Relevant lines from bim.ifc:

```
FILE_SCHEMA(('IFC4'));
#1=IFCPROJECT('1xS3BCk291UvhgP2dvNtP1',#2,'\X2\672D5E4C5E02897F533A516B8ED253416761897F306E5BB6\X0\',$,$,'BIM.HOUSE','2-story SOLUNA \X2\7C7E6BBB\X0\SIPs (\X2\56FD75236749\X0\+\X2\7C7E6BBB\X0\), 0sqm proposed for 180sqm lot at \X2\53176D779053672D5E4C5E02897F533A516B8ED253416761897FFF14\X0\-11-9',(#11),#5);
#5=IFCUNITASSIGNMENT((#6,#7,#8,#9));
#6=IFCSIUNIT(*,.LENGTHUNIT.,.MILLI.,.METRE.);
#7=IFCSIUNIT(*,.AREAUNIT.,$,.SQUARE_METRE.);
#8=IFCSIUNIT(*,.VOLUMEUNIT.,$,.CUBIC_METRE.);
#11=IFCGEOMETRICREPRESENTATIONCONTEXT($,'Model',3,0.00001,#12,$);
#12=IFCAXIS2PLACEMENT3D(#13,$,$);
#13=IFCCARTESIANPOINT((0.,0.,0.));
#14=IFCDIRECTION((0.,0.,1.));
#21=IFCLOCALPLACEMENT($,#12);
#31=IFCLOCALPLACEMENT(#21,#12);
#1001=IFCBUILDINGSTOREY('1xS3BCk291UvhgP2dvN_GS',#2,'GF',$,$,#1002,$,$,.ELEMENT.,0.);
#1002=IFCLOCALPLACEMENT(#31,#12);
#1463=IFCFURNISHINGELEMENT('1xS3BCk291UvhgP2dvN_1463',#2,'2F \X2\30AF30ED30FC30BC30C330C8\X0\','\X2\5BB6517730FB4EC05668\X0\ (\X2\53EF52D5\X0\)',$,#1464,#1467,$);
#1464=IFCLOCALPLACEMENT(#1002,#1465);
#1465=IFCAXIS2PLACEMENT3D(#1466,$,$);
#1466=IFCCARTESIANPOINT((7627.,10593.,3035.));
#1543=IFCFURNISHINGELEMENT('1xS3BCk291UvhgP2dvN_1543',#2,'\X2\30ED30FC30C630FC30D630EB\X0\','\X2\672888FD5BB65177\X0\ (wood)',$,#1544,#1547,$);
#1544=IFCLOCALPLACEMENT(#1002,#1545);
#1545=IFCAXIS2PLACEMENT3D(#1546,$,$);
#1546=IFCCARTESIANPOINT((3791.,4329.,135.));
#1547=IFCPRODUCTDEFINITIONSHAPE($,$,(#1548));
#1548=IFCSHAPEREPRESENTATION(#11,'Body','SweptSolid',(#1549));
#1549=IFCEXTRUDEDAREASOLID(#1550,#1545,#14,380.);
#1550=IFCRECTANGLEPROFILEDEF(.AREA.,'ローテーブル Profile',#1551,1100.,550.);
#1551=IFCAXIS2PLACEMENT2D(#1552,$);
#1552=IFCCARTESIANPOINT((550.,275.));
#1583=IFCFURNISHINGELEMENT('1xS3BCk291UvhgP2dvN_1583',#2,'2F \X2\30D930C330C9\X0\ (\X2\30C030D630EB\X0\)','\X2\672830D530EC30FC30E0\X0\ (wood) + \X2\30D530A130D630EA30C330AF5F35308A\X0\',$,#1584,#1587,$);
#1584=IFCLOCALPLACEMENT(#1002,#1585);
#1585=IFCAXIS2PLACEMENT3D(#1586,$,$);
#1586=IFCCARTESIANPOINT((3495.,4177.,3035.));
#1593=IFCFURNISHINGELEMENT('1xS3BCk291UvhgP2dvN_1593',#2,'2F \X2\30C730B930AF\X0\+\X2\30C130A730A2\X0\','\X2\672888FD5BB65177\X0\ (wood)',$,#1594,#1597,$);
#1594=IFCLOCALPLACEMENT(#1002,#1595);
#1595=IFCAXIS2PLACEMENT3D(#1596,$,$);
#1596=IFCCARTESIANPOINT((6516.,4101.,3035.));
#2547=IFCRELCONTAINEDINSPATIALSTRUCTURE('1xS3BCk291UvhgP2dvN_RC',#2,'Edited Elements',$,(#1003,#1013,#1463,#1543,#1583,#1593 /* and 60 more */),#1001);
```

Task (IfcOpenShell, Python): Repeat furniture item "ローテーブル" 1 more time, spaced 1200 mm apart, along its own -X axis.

```python
import ifcopenshell
import ifcopenshell.api.geometry
import ifcopenshell.api.root
import ifcopenshell.util.element
import ifcopenshell.util.placement
import ifcopenshell.util.unit

model = ifcopenshell.open("bim.ifc")
unit_scale = ifcopenshell.util.unit.calculate_unit_scale(model)


def reuse_history(source, copy):
    """copy_class also copies each property set's owner history, people and application; keep the originals."""
    for rel in copy.IsDefinedBy:
        if rel.is_a("IfcRelDefinesByProperties") and (history := rel.RelatingPropertyDefinition.OwnerHistory):
            rel.RelatingPropertyDefinition.OwnerHistory = source.OwnerHistory
            ifcopenshell.util.element.remove_deep2(model, history)


source = model.by_guid("1xS3BCk291UvhgP2dvN_1543")
base = ifcopenshell.util.placement.get_local_placement(source.ObjectPlacement)
step = -base[:3, 0] * 1.2 / unit_scale

for i in range(1, 2):
    copy = ifcopenshell.api.root.copy_class(model, product=source)
    copy.Representation = ifcopenshell.util.element.copy_deep(
        model, source.Representation, exclude=["IfcGeometricRepresentationContext", "IfcRepresentationMap"]
    )
    reuse_history(source, copy)
    matrix = base.copy()
    matrix[:3, 3] += i * step
    print("added at", matrix[:3, 3].round(3) + 0.0)
    ifcopenshell.api.geometry.edit_object_placement(model, product=copy, matrix=matrix, is_si=False)

model.write("bim_updated.ifc")
```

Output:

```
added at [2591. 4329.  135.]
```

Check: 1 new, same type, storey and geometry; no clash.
